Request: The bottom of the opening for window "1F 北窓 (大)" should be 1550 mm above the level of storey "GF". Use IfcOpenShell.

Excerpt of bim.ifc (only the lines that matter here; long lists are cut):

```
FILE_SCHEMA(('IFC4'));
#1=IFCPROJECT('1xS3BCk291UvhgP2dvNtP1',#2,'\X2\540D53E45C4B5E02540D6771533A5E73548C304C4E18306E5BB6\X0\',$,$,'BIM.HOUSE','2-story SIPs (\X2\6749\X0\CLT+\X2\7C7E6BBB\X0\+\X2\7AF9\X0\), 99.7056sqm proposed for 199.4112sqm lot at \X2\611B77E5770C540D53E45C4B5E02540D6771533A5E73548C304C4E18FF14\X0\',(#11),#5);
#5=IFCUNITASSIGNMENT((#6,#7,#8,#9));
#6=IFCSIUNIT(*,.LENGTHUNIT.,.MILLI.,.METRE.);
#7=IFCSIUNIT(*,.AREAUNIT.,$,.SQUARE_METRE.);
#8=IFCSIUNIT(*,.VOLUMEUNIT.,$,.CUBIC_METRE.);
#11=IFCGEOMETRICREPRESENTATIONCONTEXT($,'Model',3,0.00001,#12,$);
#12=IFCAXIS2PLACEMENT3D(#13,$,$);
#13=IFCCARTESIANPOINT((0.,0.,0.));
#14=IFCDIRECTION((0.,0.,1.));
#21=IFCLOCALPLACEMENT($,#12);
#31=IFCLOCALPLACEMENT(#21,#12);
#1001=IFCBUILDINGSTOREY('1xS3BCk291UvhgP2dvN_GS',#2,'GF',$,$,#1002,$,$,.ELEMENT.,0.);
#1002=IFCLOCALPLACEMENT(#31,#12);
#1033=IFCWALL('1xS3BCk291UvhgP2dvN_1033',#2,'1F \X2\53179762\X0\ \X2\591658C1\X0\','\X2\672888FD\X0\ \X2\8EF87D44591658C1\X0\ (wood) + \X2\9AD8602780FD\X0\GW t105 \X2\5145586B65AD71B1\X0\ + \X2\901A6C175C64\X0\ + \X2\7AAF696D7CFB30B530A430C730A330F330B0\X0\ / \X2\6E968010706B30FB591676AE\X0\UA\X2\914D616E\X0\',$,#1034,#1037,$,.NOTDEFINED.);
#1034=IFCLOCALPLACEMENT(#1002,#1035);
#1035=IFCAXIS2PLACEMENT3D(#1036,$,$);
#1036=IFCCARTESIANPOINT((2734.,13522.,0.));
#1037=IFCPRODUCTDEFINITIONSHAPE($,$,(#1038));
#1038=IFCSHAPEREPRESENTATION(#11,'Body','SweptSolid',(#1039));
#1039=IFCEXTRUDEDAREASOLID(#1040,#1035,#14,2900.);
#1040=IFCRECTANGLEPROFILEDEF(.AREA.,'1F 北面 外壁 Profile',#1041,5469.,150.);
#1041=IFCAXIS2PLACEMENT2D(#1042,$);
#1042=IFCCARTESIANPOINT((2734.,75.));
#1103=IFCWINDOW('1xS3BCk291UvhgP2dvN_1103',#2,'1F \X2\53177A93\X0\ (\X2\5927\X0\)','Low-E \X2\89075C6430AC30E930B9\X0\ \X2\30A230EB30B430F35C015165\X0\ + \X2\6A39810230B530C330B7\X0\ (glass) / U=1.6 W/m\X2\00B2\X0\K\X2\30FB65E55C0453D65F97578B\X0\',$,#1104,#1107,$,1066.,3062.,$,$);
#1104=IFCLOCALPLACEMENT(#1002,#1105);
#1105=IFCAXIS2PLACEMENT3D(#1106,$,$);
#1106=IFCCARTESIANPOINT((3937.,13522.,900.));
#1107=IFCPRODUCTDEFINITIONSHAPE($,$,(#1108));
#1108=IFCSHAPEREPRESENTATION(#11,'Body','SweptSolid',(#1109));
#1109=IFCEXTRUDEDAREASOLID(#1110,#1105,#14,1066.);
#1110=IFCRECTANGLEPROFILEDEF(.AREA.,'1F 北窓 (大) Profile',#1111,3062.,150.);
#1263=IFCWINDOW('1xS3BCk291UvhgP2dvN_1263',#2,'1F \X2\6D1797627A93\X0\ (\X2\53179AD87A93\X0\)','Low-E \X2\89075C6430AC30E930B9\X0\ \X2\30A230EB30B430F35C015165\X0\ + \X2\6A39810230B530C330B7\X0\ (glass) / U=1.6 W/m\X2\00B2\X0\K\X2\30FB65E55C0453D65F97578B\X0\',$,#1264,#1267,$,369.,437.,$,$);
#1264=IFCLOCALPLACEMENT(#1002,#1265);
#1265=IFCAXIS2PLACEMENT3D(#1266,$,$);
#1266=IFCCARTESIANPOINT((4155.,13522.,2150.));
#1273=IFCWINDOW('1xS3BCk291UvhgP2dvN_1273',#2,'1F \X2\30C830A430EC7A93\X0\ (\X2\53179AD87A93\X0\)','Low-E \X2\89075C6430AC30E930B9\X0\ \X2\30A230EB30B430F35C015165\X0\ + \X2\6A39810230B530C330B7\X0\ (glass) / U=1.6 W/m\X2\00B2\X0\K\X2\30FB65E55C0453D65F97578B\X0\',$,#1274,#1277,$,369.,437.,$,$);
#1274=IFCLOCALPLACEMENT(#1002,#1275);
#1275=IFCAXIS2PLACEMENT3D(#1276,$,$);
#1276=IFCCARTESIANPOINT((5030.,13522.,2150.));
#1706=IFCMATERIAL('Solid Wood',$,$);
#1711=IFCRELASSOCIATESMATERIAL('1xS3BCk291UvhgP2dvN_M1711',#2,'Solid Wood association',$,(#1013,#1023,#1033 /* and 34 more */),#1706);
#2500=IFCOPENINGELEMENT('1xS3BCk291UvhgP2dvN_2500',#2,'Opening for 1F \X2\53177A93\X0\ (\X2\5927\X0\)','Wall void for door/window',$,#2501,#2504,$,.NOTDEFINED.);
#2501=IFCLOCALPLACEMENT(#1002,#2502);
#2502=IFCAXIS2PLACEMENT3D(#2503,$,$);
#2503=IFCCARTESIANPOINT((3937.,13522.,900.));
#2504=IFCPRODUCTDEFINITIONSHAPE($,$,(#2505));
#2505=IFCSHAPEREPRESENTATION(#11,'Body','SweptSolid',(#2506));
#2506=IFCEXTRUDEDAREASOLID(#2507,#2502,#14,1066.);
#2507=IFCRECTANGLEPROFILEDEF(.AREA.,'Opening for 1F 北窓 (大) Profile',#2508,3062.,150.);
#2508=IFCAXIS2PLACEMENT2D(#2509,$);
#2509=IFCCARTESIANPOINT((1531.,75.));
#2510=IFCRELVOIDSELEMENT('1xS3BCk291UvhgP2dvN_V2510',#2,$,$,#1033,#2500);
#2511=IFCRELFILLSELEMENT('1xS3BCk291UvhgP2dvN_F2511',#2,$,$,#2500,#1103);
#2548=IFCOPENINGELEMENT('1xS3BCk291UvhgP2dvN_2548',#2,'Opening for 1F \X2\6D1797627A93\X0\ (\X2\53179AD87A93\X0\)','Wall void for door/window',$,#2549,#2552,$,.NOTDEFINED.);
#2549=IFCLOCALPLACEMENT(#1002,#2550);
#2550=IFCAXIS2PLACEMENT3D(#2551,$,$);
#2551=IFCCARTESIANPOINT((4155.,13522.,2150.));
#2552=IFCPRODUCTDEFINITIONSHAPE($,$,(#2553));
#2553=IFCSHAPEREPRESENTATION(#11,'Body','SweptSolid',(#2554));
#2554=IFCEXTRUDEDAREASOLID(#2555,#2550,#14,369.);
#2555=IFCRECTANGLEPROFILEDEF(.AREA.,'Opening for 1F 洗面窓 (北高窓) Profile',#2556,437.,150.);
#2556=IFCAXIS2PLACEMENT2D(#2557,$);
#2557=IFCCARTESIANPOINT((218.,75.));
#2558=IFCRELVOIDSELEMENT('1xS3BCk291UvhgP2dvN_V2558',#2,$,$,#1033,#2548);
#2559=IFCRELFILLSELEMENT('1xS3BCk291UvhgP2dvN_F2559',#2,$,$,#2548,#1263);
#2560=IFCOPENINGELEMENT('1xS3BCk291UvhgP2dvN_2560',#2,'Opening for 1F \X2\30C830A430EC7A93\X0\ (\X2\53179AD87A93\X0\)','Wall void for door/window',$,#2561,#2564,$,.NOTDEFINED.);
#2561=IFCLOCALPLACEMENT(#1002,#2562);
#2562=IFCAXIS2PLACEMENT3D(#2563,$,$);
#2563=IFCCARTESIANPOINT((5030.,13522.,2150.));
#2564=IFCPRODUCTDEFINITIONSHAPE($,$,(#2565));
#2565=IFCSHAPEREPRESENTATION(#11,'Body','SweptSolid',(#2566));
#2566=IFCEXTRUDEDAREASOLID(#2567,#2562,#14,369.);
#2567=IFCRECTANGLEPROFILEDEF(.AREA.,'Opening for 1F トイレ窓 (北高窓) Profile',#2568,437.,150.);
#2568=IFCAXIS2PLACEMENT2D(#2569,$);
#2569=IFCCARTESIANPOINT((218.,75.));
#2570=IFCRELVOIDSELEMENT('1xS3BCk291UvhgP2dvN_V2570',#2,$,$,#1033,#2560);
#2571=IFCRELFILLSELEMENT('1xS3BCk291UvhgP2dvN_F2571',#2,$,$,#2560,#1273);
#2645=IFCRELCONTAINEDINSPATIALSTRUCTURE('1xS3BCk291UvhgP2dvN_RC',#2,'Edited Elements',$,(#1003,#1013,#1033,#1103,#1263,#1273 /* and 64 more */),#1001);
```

```python
import numpy as np
import ifcopenshell
import ifcopenshell.api.geometry
import ifcopenshell.geom
import ifcopenshell.util.element
import ifcopenshell.util.placement
import ifcopenshell.util.shape
import ifcopenshell.util.unit

model = ifcopenshell.open("bim.ifc")
unit_scale = ifcopenshell.util.unit.calculate_unit_scale(model)

window = model.by_id(1103)
opening = window.FillsVoids[0].RelatingOpeningElement
storey = ifcopenshell.util.element.get_container(window, ifc_class="IfcBuildingStorey")
level = ifcopenshell.util.placement.get_local_placement(storey.ObjectPlacement)[2, 3]

# The opening's origin need not be at the sill, so measure its lowest point.
shape = ifcopenshell.geom.create_shape(ifcopenshell.geom.settings(), opening)
bottom = ifcopenshell.util.shape.get_shape_bottom_elevation(shape, shape.geometry) / unit_scale
dz = level + 1.55 / unit_scale - bottom

shift = np.array([0.0, 0.0, dz])
# The window is not placed relative to its opening, so move both.
for product in (opening, window):
    matrix = ifcopenshell.util.placement.get_local_placement(product.ObjectPlacement)
    matrix[:3, 3] += shift
    ifcopenshell.api.geometry.edit_object_placement(model, product=product, matrix=matrix, is_si=False)

print(f"moved by {dz * unit_scale:+.3f} m")

model.write("bim_edited.ifc")
```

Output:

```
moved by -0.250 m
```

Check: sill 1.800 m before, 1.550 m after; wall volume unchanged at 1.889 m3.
